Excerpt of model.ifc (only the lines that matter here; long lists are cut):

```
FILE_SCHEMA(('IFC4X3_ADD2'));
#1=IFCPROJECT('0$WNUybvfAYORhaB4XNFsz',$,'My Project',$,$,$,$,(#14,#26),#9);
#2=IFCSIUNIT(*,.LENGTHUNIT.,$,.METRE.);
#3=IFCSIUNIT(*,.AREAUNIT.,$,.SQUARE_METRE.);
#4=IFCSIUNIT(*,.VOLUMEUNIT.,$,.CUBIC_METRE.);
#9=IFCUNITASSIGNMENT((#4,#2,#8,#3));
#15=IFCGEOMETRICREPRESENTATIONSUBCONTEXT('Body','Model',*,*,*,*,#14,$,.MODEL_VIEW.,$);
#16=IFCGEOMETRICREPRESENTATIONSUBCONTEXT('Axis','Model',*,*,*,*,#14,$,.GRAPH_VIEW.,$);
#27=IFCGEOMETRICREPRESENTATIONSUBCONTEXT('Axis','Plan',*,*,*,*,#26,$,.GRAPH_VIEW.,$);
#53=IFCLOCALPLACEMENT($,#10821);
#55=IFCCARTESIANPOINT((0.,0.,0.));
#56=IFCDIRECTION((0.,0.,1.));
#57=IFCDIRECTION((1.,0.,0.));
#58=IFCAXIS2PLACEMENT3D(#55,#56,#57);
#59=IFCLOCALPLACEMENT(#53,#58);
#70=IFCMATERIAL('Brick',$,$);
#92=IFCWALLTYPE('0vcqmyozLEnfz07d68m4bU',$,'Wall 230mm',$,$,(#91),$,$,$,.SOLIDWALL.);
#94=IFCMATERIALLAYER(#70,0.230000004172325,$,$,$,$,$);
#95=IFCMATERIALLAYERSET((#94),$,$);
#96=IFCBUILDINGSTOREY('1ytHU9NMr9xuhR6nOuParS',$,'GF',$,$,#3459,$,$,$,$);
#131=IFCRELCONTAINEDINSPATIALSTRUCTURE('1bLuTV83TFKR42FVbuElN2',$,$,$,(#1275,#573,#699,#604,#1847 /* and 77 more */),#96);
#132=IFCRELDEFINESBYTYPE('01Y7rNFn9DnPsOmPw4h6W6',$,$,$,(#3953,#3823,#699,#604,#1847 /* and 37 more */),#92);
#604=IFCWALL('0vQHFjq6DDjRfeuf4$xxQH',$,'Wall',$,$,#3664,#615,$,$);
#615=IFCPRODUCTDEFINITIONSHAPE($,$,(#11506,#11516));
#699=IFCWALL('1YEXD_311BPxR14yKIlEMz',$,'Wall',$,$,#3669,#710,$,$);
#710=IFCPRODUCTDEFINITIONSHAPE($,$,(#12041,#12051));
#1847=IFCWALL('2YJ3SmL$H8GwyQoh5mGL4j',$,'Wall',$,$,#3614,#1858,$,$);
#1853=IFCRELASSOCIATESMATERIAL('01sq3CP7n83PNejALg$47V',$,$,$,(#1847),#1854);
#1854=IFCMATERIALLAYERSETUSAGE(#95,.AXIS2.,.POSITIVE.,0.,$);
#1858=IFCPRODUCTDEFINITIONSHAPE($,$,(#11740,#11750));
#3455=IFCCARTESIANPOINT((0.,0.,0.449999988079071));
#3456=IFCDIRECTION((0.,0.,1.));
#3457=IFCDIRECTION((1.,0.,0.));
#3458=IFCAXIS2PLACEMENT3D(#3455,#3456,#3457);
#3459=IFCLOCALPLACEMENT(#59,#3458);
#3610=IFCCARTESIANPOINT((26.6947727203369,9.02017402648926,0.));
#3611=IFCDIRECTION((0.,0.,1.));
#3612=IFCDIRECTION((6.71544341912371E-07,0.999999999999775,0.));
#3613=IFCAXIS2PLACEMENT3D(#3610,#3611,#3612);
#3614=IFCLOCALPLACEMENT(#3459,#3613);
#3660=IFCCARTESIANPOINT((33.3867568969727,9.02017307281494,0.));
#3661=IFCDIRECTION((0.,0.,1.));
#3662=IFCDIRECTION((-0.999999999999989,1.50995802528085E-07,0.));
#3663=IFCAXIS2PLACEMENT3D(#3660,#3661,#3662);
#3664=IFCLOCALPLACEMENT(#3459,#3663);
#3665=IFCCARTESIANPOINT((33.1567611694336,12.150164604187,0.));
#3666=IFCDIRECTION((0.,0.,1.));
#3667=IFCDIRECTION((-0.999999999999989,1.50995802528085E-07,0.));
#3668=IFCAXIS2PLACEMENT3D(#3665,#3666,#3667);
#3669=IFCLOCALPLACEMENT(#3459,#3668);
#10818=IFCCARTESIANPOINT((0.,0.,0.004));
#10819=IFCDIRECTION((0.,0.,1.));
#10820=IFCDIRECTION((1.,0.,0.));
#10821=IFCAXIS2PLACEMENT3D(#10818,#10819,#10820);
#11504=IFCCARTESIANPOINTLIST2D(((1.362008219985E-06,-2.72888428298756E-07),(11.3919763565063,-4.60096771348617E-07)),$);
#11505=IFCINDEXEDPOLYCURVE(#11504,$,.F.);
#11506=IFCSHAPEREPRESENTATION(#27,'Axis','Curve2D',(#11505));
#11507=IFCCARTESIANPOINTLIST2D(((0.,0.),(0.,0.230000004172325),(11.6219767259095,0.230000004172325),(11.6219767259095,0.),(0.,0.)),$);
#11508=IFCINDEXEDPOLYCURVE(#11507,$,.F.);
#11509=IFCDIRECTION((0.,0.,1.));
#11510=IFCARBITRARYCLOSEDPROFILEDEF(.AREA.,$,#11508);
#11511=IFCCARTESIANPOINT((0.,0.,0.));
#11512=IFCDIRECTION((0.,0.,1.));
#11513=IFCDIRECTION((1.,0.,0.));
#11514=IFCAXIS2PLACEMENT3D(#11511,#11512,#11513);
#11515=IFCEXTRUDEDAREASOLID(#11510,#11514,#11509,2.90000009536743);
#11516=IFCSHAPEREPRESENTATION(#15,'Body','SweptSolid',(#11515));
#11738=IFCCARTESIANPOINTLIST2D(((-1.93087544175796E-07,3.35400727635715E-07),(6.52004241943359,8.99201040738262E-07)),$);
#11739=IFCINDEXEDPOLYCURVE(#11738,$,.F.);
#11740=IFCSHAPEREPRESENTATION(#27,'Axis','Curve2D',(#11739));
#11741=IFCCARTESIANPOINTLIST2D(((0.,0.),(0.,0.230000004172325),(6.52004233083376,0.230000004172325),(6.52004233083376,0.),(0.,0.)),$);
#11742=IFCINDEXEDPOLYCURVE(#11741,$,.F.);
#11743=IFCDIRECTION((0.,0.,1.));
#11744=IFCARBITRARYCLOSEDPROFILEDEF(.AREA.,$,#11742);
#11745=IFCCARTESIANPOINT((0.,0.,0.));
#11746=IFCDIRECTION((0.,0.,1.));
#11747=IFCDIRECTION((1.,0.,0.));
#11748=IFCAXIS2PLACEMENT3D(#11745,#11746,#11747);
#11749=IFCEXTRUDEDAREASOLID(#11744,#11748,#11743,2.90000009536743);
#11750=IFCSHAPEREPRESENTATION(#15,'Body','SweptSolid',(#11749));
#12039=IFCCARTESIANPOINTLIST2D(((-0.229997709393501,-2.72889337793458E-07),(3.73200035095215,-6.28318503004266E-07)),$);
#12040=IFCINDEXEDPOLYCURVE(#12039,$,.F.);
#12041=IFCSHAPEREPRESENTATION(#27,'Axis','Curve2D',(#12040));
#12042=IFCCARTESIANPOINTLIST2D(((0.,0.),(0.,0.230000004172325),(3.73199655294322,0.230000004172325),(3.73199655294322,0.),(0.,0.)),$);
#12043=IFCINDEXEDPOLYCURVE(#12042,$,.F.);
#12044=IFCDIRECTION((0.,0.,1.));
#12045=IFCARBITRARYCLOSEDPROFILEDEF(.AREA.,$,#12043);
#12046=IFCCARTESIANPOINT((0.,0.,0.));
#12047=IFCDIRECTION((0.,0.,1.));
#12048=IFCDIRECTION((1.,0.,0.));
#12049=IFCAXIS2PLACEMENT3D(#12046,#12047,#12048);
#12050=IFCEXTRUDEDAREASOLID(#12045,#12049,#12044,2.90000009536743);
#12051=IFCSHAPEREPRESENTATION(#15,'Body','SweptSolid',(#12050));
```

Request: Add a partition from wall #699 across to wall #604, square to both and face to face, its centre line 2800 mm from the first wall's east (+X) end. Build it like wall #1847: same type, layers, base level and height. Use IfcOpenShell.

```python
import numpy as np
import ifcopenshell
import ifcopenshell.api.geometry
import ifcopenshell.api.material
import ifcopenshell.api.pset
import ifcopenshell.api.root
import ifcopenshell.api.spatial
import ifcopenshell.api.type
import ifcopenshell.geom
import ifcopenshell.util.element
import ifcopenshell.util.placement
import ifcopenshell.util.representation
import ifcopenshell.util.shape
import ifcopenshell.util.unit

model = ifcopenshell.open("model.ifc")
unit_scale = ifcopenshell.util.unit.calculate_unit_scale(model)
settings = ifcopenshell.geom.settings()
settings.set("use-world-coords", True)

start_wall = model.by_id(699)
end_wall = model.by_guid("0vQHFjq6DDjRfeuf4$xxQH")
like = model.by_guid("2YJ3SmL$H8GwyQoh5mGL4j")
matrix = ifcopenshell.util.placement.get_local_placement(start_wall.ObjectPlacement)
matrix[:3, 3] *= unit_scale


def extent(element):
    """Bounding box in the first wall's axes, in metres."""
    shape = ifcopenshell.geom.create_shape(settings, element)
    points = (ifcopenshell.util.shape.get_vertices(shape.geometry) - matrix[:3, 3]) @ matrix[:3, :3]
    return points.min(axis=0), points.max(axis=0)


y_start = extent(start_wall)[1][1]
y_end = extent(end_wall)[0][1]
like_min, like_max = extent(like)
length, height = float(abs(y_end - y_start)), float(like_max[2] - like_min[2])
layer_set = ifcopenshell.util.element.get_material(like, should_skip_usage=True)
thickness = sum(layer.LayerThickness for layer in layer_set.MaterialLayers) * unit_scale

wall = ifcopenshell.api.root.create_entity(model, ifc_class="IfcWall", name="New partition")
storey = ifcopenshell.util.element.get_container(like)
ifcopenshell.api.spatial.assign_container(model, products=[wall], relating_structure=storey)
ifcopenshell.api.type.assign_type(
    model, related_objects=[wall], relating_type=ifcopenshell.util.element.get_type(like), should_map_representations=False
)
rel = ifcopenshell.api.material.assign_material(
    model, products=[wall], type="IfcMaterialLayerSetUsage", material=layer_set
)
rel.RelatingMaterial.OffsetFromReferenceLine = -thickness / 2 / unit_scale
pset = ifcopenshell.api.pset.add_pset(model, product=wall, name="Pset_WallCommon")
ifcopenshell.api.pset.edit_pset(model, pset=pset, properties={"IsExternal": False, "LoadBearing": False})

# The axis runs down the middle of the wall.
axis = ifcopenshell.api.geometry.add_axis_representation(
    model, context=ifcopenshell.util.representation.get_context(model, "Model", "Axis"), axis=[(0.0, 0.0), (length, 0.0)]
)
body = ifcopenshell.api.geometry.add_wall_representation(
    model,
    context=ifcopenshell.util.representation.get_context(model, "Model", "Body", "MODEL_VIEW"),
    length=length,
    height=height,
    thickness=thickness,
    offset=-thickness / 2,
)
for representation in (axis, body):
    ifcopenshell.api.geometry.assign_representation(model, product=wall, representation=representation)

placement = matrix @ ifcopenshell.util.placement.rotation(90, "Z")
placement[:, 3] = matrix @ np.array([extent(start_wall)[0][0] + 2.8, y_start, like_min[2], 1.0])
ifcopenshell.api.geometry.edit_object_placement(model, product=wall, matrix=placement)

print(f"partition {length:.3f} m long, {height:.3f} m high, {thickness:.3f} m thick")

model.write("model_edited.ifc")
```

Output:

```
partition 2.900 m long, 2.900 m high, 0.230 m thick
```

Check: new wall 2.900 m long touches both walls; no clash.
